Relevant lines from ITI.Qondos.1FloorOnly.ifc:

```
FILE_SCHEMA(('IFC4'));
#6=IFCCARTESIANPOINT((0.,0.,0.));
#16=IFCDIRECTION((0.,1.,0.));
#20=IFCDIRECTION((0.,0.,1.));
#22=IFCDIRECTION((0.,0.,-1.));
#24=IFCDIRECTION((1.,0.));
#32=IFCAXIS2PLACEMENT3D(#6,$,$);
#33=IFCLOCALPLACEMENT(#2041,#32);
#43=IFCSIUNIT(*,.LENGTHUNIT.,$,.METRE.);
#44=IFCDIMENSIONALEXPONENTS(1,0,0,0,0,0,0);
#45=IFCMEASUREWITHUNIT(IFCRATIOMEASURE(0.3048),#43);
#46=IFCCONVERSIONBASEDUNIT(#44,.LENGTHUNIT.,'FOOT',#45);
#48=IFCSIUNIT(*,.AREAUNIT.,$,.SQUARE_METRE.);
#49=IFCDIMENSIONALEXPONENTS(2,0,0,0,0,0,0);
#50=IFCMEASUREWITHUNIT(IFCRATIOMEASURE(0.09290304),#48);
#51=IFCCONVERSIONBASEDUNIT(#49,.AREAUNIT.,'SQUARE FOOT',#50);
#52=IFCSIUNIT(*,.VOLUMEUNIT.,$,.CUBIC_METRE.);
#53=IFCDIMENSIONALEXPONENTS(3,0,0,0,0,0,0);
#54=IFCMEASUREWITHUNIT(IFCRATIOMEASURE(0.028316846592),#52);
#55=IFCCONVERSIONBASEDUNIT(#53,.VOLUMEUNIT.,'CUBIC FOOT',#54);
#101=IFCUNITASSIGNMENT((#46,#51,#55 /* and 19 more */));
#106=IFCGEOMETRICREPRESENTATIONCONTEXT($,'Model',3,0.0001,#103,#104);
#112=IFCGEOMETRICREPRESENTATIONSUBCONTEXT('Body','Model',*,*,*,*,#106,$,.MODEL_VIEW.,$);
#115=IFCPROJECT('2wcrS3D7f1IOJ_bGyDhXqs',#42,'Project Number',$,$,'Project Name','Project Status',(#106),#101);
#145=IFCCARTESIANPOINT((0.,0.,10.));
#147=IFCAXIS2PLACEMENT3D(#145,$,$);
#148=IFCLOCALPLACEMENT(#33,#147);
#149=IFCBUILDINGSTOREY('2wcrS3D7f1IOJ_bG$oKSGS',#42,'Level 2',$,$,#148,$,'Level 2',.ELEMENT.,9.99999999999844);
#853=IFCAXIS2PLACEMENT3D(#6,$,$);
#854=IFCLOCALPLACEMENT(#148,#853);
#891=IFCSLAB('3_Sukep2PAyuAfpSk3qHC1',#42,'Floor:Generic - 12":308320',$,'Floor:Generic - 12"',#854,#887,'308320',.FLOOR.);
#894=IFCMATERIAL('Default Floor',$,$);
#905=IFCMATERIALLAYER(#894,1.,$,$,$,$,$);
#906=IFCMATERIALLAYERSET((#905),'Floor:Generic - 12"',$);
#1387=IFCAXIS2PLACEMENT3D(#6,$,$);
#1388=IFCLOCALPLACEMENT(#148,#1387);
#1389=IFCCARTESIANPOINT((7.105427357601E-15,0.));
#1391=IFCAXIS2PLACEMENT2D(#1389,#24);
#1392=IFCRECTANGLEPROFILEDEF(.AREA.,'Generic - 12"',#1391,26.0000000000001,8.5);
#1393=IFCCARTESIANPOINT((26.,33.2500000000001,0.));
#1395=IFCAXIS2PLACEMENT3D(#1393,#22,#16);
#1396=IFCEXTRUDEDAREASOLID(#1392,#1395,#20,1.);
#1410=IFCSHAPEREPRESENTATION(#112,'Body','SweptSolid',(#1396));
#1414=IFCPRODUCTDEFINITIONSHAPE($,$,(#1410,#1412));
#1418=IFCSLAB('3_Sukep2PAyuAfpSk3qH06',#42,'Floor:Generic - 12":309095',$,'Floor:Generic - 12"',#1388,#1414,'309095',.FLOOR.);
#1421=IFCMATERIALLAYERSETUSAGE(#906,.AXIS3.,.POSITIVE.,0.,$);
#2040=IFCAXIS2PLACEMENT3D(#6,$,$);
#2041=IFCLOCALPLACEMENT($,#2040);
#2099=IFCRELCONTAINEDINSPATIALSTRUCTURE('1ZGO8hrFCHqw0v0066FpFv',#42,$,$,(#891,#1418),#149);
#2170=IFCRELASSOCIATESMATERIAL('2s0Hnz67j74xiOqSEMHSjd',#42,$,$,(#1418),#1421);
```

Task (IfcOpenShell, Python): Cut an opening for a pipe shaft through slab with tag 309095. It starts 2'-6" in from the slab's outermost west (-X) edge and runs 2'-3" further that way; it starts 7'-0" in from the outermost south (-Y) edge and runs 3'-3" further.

```python
import numpy as np
import ifcopenshell
import ifcopenshell.api.feature
import ifcopenshell.api.geometry
import ifcopenshell.api.root
import ifcopenshell.geom
import ifcopenshell.util.placement
import ifcopenshell.util.representation
import ifcopenshell.util.shape
import ifcopenshell.util.unit

model = ifcopenshell.open("ITI.Qondos.1FloorOnly.ifc")
unit_scale = ifcopenshell.util.unit.calculate_unit_scale(model)
settings = ifcopenshell.geom.settings()


def volume(element):
    """Net volume in cubic metres, openings subtracted."""
    shape = ifcopenshell.geom.create_shape(settings, element)
    return ifcopenshell.util.shape.get_volume(shape.geometry)


slab = model.by_guid("3_Sukep2PAyuAfpSk3qH06")
before = volume(slab)

# Extent in the slab's own axes, in metres. The edges named are its -X and -Y sides.
slab_shape = ifcopenshell.geom.create_shape(settings, slab)
vertices = ifcopenshell.util.shape.get_vertices(slab_shape.geometry)
x_min, y_min, bottom = vertices.min(axis=0)
top = vertices[:, 2].max()

opening = ifcopenshell.api.root.create_entity(model, ifc_class="IfcOpeningElement", name="Pipe shaft opening", predefined_type="OPENING")
context = ifcopenshell.util.representation.get_context(model, "Model", "Body", "MODEL_VIEW")
width, depth = 0.6858, 0.9906
outline = [(0.0, 0.0), (width, 0.0), (width, depth), (0.0, depth), (0.0, 0.0)]
# Overshoot both faces by 50 mm so the cut is clean.
shape = ifcopenshell.api.geometry.add_slab_representation(
    model, context=context, depth=top - bottom + 0.1, polyline=outline
)
ifcopenshell.api.geometry.assign_representation(model, product=opening, representation=shape)

matrix = ifcopenshell.util.placement.get_local_placement(slab.ObjectPlacement)
matrix[:, 3] = matrix @ np.append(np.array([x_min + 0.762, y_min + 2.1336, bottom - 0.05]) / unit_scale, 1.0)
ifcopenshell.api.geometry.edit_object_placement(model, product=opening, matrix=matrix, is_si=False)
ifcopenshell.api.feature.add_feature(model, feature=opening, element=slab)

after = volume(slab)

print(f"slab volume {before:.3f} -> {after:.3f} m3")

model.write("ITI.Qondos.1FloorOnly_updated.ifc")
```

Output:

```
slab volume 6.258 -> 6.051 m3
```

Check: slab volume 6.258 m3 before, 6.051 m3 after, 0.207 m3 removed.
